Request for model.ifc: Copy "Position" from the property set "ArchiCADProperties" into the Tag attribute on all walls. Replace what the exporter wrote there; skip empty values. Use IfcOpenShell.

First a look at what the model holds.

```python
import ifcopenshell
import ifcopenshell.util.element

model = ifcopenshell.open("model.ifc")
print(model.schema)
walls = model.by_type("IfcWall")
print(len(walls), "walls")
for e in walls[:8]:
    source = ifcopenshell.util.element.get_pset(e, "ArchiCADProperties", "Position")
    target = e.Tag
    print(e.id(), repr(source), repr(target), sep=" | ")
```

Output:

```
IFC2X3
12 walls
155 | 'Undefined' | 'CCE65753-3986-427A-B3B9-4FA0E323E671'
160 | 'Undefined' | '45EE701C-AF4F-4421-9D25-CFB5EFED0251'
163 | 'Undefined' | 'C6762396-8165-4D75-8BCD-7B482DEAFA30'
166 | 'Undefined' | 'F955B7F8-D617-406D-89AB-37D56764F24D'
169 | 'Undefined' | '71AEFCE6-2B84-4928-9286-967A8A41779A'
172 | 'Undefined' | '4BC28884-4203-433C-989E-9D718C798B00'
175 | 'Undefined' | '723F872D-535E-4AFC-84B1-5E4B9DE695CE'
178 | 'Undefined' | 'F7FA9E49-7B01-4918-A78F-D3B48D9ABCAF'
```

```python
import ifcopenshell
import ifcopenshell.util.element

model = ifcopenshell.open("model.ifc")

count = 0
for e in model.by_type("IfcWall"):
    value = ifcopenshell.util.element.get_pset(e, "ArchiCADProperties", "Position")
    current = e.Tag
    if not value or not value.strip() or current == value:
        continue
    e.Tag = value
    count += 1

print(count, "walls updated")

model.write("model_rev.ifc")
```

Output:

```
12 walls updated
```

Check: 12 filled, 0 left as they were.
